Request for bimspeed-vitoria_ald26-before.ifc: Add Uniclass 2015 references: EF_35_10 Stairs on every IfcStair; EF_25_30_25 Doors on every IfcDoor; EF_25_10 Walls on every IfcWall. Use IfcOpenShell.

First a look at what the model holds.

```python
import ifcopenshell

model = ifcopenshell.open("bimspeed-vitoria_ald26-before.ifc")
print(model.schema)
print("classifications:", [c.Name for c in model.by_type("IfcClassification")])
for ifc_class in ("IfcDoor", "IfcRoof", "IfcStair", "IfcWall", "IfcWindow"):
    print(ifc_class, len(model.by_type(ifc_class)))
```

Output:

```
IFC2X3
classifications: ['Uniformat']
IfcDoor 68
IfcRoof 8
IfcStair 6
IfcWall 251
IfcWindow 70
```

```python
import ifcopenshell
import ifcopenshell.api.classification

model = ifcopenshell.open("bimspeed-vitoria_ald26-before.ifc")

# IFC2X3 requires Source and Edition and has no link from the project to the system.
system = model.create_entity("IfcClassification", Source="NBS", Edition="2015", Name="Uniclass 2015")

codes = {
    "IfcStair": ("EF_35_10", "Stairs"),
    "IfcDoor": ("EF_25_30_25", "Doors"),
    "IfcWall": ("EF_25_10", "Walls"),
}
for ifc_class, (code, name) in codes.items():
    products = model.by_type(ifc_class)
    ifcopenshell.api.classification.add_reference(
        model, products=products, classification=system, identification=code, name=name
    )
    print(code, len(products))

model.write("bimspeed-vitoria_ald26-before-out.ifc")
```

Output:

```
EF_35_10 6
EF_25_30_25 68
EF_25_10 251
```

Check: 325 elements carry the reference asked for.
